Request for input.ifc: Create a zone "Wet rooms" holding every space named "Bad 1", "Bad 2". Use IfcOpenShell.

First a look at what the model holds.

```python
import ifcopenshell

model = ifcopenshell.open("input.ifc")
print(model.schema)
seen = {}
for space in model.by_type("IfcSpace"):
    seen[space.LongName] = seen.get(space.LongName, 0) + 1
for name, count in sorted(seen.items(), key=str):
    print(count, "x", name)
print("zones:", [z.Name for z in model.by_type("IfcZone")][:20])
```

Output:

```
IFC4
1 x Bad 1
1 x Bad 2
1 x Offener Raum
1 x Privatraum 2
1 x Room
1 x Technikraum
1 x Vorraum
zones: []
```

```python
import ifcopenshell
import ifcopenshell.api.group
import ifcopenshell.api.root

model = ifcopenshell.open("input.ifc")

names = {"Bad 1", "Bad 2"}
spaces = [s for s in model.by_type("IfcSpace") if s.LongName in names]

zone = ifcopenshell.api.root.create_entity(model, ifc_class="IfcZone", name="Wet rooms")
ifcopenshell.api.group.assign_group(model, products=spaces, group=zone)
print(len(spaces), "spaces in", zone.Name)

model.write("input_edited.ifc")
```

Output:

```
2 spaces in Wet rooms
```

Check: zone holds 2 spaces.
